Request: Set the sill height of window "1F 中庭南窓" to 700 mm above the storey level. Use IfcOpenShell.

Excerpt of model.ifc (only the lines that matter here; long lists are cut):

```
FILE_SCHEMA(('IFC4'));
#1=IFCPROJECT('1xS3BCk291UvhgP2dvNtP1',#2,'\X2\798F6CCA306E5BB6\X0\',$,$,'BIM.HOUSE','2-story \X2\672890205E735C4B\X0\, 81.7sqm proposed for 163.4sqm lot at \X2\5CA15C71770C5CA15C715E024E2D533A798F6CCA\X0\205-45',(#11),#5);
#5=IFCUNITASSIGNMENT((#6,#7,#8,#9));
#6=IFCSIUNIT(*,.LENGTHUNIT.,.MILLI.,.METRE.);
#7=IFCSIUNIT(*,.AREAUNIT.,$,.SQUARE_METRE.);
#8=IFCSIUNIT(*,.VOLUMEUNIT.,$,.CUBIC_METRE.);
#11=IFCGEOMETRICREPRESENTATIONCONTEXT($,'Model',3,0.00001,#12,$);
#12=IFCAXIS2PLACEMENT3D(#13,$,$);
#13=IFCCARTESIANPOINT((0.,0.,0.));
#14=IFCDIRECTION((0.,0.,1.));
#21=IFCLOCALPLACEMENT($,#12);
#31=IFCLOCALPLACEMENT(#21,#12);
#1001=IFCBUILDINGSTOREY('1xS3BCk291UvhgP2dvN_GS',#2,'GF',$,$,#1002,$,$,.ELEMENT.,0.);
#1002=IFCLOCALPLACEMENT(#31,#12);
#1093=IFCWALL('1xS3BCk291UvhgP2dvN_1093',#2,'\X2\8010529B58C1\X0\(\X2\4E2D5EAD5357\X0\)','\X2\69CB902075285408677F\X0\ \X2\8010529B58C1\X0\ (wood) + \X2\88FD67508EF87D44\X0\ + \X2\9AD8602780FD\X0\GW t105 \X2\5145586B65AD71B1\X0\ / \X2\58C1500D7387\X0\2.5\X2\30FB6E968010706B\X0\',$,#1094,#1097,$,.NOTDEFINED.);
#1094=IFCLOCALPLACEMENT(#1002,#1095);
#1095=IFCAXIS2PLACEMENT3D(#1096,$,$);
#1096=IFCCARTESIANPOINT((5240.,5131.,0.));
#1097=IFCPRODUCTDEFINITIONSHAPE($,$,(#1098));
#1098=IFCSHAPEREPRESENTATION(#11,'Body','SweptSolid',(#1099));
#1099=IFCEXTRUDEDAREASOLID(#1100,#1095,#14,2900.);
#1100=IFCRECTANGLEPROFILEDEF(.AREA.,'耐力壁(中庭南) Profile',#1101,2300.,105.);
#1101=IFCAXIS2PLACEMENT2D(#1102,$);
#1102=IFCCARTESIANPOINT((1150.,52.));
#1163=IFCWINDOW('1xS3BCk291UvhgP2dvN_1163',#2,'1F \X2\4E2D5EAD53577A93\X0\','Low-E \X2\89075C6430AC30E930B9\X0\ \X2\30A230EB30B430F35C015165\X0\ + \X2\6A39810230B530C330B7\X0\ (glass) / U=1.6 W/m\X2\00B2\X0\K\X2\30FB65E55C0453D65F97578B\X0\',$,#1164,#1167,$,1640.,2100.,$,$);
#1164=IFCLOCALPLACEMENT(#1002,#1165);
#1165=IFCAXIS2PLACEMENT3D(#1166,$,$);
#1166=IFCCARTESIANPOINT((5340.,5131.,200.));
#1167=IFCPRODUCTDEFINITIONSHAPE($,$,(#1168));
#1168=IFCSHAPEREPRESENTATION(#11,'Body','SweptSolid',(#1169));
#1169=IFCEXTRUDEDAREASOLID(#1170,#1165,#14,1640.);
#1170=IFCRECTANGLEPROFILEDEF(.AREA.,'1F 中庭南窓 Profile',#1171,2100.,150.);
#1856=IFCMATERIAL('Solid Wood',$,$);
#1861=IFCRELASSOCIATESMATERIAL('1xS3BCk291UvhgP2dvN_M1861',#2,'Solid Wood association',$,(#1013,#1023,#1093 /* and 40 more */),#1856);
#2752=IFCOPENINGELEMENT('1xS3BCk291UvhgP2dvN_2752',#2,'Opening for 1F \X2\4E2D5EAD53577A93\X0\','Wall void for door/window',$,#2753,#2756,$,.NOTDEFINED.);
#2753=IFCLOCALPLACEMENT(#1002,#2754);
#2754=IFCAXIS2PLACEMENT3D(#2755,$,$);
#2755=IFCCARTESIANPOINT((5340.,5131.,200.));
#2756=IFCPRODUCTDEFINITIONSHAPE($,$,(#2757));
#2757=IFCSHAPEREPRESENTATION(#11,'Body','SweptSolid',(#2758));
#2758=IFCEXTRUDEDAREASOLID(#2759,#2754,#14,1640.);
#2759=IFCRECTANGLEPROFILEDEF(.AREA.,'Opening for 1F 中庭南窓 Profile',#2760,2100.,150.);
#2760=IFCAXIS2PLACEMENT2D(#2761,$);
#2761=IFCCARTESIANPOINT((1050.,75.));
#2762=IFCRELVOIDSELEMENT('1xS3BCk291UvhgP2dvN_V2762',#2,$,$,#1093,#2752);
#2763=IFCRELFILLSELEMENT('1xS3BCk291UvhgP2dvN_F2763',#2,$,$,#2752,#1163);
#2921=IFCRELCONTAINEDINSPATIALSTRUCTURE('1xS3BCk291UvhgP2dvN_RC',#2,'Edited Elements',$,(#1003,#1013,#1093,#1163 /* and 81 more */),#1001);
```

```python
import numpy as np
import ifcopenshell
import ifcopenshell.api.geometry
import ifcopenshell.geom
import ifcopenshell.util.element
import ifcopenshell.util.placement
import ifcopenshell.util.shape
import ifcopenshell.util.unit

model = ifcopenshell.open("model.ifc")
unit_scale = ifcopenshell.util.unit.calculate_unit_scale(model)

window = model.by_guid("1xS3BCk291UvhgP2dvN_1163")
opening = window.FillsVoids[0].RelatingOpeningElement
storey = ifcopenshell.util.element.get_container(window, ifc_class="IfcBuildingStorey")
level = ifcopenshell.util.placement.get_local_placement(storey.ObjectPlacement)[2, 3]

# The opening's origin need not be at the sill, so measure its lowest point.
shape = ifcopenshell.geom.create_shape(ifcopenshell.geom.settings(), opening)
bottom = ifcopenshell.util.shape.get_shape_bottom_elevation(shape, shape.geometry) / unit_scale
dz = level + 0.7 / unit_scale - bottom

shift = np.array([0.0, 0.0, dz])
# The window is not placed relative to its opening, so move both.
for product in (opening, window):
    matrix = ifcopenshell.util.placement.get_local_placement(product.ObjectPlacement)
    matrix[:3, 3] += shift
    ifcopenshell.api.geometry.edit_object_placement(model, product=product, matrix=matrix, is_si=False)

print(f"moved by {dz * unit_scale:+.3f} m")

model.write("model-out.ifc")
```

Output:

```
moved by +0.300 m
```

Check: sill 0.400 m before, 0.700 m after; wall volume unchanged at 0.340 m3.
